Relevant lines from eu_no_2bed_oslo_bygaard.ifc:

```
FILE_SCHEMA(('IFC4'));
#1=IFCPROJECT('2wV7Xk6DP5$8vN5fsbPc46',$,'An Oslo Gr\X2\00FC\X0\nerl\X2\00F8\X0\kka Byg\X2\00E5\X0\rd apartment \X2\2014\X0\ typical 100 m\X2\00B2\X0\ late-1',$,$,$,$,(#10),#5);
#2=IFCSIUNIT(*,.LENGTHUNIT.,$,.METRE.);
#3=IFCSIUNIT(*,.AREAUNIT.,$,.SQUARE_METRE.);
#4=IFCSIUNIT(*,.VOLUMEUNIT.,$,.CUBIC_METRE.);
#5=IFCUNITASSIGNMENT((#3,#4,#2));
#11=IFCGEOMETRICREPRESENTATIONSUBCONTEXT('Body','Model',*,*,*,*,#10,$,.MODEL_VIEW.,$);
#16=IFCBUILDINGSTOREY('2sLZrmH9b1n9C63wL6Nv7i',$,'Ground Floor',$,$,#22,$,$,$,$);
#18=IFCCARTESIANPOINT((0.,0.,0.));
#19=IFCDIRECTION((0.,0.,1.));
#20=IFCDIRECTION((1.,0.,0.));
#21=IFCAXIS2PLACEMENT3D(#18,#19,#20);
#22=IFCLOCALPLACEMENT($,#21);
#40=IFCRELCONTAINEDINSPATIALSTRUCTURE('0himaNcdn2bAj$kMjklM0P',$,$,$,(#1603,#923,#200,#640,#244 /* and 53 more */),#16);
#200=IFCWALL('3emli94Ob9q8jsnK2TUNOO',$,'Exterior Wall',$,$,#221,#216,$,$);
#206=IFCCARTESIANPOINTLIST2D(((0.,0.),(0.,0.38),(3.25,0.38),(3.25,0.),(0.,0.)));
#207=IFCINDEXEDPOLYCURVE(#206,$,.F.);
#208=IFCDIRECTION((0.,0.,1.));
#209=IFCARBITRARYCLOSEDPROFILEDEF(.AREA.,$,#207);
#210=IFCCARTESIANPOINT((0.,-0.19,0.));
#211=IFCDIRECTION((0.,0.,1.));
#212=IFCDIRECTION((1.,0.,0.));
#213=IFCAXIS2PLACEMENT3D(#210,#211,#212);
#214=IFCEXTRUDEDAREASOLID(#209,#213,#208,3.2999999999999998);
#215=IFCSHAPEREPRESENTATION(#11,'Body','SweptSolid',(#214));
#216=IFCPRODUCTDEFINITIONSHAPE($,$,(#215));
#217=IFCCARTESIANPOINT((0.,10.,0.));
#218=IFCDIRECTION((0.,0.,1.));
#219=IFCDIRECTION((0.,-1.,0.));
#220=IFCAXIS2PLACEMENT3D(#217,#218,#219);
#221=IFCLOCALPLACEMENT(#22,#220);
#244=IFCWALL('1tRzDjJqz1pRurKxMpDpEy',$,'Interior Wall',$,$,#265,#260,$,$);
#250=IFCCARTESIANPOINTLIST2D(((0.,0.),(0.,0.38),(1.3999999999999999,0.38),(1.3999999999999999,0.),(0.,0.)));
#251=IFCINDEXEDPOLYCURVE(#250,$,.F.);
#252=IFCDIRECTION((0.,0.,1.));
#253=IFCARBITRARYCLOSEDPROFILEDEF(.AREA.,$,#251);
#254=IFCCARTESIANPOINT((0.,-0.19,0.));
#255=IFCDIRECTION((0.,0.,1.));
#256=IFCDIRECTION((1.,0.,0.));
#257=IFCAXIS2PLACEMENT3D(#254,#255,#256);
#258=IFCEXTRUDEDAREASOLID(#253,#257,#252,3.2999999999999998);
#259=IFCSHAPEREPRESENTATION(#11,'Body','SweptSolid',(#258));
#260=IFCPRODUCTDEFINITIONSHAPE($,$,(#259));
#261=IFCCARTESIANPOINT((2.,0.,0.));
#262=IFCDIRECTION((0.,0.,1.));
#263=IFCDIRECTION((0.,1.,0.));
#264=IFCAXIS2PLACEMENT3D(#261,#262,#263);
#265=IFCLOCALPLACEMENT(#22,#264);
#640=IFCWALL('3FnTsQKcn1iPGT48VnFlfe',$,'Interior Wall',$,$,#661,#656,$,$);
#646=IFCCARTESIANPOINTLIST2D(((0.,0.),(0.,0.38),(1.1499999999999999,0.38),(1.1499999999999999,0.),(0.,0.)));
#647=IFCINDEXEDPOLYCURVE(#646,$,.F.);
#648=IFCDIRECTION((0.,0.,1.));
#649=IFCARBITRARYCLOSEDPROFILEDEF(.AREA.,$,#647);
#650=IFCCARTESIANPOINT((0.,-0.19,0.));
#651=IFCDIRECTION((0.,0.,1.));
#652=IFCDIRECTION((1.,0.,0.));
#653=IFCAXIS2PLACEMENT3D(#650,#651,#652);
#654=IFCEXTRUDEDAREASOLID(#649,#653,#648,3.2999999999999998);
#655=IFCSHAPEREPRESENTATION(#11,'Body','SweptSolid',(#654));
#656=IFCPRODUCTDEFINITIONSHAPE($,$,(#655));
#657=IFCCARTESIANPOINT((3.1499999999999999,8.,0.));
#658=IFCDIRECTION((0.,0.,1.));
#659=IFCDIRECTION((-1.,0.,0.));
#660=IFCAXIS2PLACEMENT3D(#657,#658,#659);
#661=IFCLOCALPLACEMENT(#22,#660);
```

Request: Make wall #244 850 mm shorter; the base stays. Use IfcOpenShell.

```python
import ifcopenshell
import ifcopenshell.geom
import ifcopenshell.util.representation
import ifcopenshell.util.shape

model = ifcopenshell.open("eu_no_2bed_oslo_bygaard.ifc")
settings = ifcopenshell.geom.settings()


def volume(element):
    """Net volume in cubic metres, openings subtracted."""
    shape = ifcopenshell.geom.create_shape(settings, element)
    return ifcopenshell.util.shape.get_volume(shape.geometry)


wall = model.by_guid("1tRzDjJqz1pRurKxMpDpEy")
before = volume(wall)

body = ifcopenshell.util.representation.get_representation(wall, "Model", "Body")
solid = body.Items[0]
old_height = solid.Depth
solid.Depth -= 0.85
after = volume(wall)

print(f"height {old_height:g} -> {solid.Depth:g}, volume {before:.3f} -> {after:.3f} m3")

model.write("eu_no_2bed_oslo_bygaard_updated.ifc")
```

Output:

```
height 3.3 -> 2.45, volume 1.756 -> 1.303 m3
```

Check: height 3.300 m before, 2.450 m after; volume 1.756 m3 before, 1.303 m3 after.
